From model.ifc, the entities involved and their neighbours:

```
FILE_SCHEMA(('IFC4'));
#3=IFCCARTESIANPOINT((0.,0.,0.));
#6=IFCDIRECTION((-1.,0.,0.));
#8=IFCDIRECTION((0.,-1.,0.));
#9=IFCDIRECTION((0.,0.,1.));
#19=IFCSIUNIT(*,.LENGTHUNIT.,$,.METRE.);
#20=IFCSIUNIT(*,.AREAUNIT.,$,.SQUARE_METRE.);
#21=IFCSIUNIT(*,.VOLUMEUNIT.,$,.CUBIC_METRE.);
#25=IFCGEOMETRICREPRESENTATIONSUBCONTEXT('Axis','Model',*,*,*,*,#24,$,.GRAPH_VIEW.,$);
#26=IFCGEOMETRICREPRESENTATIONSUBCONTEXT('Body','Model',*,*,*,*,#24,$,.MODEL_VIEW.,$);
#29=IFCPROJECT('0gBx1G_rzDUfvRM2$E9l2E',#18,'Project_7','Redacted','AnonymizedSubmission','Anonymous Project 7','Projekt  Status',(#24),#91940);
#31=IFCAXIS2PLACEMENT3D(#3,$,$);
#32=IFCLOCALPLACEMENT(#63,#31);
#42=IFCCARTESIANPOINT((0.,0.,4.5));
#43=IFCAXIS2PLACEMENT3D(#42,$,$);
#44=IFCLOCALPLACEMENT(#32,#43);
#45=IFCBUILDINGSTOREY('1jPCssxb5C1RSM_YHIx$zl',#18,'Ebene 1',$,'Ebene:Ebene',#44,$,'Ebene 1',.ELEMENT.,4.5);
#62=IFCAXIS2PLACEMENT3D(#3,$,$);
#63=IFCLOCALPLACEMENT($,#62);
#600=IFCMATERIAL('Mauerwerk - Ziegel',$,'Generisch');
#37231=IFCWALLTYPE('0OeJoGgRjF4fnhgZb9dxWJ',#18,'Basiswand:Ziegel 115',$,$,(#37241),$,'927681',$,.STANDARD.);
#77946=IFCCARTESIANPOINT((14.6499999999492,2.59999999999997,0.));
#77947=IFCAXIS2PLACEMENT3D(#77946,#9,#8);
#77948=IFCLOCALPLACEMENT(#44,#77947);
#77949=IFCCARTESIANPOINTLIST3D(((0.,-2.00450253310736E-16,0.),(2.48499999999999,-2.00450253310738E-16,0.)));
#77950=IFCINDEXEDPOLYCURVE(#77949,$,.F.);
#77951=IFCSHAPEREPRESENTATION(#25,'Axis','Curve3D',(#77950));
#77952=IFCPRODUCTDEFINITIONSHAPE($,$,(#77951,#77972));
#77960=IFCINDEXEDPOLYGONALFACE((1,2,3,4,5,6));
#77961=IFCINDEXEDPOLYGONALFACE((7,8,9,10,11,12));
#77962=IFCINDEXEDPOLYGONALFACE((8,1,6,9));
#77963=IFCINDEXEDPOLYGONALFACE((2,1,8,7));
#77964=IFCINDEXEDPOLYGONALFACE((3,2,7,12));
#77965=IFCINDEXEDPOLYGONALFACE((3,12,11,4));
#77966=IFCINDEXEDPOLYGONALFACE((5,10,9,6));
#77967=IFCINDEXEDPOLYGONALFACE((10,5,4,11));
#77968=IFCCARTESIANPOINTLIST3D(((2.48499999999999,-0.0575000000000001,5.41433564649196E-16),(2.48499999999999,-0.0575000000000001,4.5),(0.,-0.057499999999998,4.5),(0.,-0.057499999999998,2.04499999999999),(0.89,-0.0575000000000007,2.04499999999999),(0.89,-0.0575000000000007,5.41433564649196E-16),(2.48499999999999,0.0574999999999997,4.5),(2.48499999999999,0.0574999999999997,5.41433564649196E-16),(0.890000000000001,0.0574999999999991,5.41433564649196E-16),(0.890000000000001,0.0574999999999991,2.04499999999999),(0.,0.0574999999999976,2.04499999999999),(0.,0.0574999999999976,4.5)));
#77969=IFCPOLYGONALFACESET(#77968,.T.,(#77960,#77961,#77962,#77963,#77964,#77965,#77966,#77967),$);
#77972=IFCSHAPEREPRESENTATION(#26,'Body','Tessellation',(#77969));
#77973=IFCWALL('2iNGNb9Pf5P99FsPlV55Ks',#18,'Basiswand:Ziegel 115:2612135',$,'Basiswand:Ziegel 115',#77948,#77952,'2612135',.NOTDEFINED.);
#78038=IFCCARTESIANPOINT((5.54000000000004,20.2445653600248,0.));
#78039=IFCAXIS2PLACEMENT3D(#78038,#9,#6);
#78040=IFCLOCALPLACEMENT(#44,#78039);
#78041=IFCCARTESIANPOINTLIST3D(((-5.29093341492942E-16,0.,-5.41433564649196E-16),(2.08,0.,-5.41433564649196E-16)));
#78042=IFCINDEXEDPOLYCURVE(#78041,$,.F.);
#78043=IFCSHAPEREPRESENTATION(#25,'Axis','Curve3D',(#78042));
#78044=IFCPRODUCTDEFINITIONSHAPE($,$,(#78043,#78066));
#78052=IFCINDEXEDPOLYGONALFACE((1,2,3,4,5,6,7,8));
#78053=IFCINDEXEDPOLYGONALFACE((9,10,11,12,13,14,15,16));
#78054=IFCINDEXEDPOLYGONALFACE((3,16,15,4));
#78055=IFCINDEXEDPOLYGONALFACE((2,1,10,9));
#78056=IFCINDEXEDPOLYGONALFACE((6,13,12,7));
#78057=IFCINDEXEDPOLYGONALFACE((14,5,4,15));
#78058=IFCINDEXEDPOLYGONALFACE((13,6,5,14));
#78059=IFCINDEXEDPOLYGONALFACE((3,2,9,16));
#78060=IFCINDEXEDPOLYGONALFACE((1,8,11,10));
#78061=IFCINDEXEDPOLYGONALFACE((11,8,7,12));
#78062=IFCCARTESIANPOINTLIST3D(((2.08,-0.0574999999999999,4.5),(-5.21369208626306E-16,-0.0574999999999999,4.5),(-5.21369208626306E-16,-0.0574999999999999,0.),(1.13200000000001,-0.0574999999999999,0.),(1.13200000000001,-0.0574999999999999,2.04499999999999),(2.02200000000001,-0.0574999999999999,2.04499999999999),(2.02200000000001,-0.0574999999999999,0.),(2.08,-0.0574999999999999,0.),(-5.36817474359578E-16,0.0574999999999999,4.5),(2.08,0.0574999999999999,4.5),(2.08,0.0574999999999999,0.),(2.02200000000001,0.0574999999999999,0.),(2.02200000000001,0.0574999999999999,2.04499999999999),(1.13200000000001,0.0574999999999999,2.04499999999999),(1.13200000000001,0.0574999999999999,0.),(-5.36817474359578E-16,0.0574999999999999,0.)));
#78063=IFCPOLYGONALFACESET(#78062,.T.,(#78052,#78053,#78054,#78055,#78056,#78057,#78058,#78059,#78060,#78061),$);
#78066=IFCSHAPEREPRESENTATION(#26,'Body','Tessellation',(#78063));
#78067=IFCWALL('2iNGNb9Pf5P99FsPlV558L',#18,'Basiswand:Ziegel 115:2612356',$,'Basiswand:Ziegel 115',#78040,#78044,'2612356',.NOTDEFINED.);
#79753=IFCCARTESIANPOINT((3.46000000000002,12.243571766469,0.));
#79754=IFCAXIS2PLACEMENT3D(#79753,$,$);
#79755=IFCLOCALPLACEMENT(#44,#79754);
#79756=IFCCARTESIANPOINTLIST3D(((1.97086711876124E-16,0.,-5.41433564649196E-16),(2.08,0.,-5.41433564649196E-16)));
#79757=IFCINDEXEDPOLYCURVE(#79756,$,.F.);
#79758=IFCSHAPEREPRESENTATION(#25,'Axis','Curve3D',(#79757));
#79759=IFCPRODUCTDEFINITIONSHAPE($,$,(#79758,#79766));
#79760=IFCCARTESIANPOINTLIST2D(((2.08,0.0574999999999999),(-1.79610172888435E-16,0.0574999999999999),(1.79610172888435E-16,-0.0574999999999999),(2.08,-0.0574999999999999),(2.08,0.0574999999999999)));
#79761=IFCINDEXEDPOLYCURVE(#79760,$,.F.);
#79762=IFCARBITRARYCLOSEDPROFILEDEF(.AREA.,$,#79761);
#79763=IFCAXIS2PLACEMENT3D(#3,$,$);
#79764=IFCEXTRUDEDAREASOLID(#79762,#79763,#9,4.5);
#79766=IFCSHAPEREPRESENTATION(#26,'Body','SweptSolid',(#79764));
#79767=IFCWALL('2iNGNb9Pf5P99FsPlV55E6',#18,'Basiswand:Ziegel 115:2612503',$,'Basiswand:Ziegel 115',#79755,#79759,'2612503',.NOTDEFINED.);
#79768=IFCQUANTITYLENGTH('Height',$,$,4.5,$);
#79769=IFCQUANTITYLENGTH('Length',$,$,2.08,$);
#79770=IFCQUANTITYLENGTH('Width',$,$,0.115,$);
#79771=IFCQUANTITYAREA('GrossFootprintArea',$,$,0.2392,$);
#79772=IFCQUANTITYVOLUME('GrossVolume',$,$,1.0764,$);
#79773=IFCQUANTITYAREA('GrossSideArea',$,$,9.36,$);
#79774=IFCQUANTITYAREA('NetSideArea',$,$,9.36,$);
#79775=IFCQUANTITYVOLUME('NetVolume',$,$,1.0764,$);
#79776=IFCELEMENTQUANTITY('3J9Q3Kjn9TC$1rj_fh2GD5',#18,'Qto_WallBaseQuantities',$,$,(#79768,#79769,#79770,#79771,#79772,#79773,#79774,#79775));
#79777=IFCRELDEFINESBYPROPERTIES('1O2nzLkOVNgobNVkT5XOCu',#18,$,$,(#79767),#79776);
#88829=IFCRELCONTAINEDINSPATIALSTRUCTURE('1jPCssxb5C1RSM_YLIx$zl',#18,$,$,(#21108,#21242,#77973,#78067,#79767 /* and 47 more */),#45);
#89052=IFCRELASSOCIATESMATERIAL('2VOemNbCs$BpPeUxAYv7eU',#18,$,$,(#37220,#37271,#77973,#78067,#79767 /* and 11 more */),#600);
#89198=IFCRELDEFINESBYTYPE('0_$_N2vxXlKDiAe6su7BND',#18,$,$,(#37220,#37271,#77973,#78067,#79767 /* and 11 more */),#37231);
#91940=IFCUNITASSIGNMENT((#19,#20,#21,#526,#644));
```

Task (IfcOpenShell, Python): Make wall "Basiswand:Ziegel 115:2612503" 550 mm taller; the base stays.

```python
import ifcopenshell
import ifcopenshell.api.pset
import ifcopenshell.geom
import ifcopenshell.util.element
import ifcopenshell.util.representation
import ifcopenshell.util.shape
import ifcopenshell.util.unit

model = ifcopenshell.open("model.ifc")
unit_scale = ifcopenshell.util.unit.calculate_unit_scale(model)
area_scale = ifcopenshell.util.unit.calculate_unit_scale(model, "AREAUNIT")
volume_scale = ifcopenshell.util.unit.calculate_unit_scale(model, "VOLUMEUNIT")
settings = ifcopenshell.geom.settings()


def volume(element):
    """Net volume in cubic metres, openings subtracted."""
    shape = ifcopenshell.geom.create_shape(settings, element)
    return ifcopenshell.util.shape.get_volume(shape.geometry)


wall = model.by_id(79767)
before = volume(wall)

body = ifcopenshell.util.representation.get_representation(wall, "Model", "Body")
solid = body.Items[0]
old_height = solid.Depth
solid.Depth += 0.55
after = volume(wall)
thickness = 0.115  # wall thickness in metres

# Update the stored height, areas and volumes.
qto = model.by_id(ifcopenshell.util.element.get_pset(wall, "Qto_WallBaseQuantities", should_inherit=False)["id"])
ifcopenshell.api.pset.edit_qto(model, qto=qto, properties={
    "Height": solid.Depth,
    "GrossVolume": ifcopenshell.util.element.get_pset(wall, "Qto_WallBaseQuantities", "GrossVolume") * solid.Depth / old_height,
    "GrossSideArea": ifcopenshell.util.element.get_pset(wall, "Qto_WallBaseQuantities", "GrossSideArea") * solid.Depth / old_height,
    "NetSideArea": after / thickness / area_scale,
    "NetVolume": after / volume_scale,
})

print(f"height {old_height:g} -> {solid.Depth:g}, volume {before:.3f} -> {after:.3f} m3")

model.write("model_v2.ifc")
```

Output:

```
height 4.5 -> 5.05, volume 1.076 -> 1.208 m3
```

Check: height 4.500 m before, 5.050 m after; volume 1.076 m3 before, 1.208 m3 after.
